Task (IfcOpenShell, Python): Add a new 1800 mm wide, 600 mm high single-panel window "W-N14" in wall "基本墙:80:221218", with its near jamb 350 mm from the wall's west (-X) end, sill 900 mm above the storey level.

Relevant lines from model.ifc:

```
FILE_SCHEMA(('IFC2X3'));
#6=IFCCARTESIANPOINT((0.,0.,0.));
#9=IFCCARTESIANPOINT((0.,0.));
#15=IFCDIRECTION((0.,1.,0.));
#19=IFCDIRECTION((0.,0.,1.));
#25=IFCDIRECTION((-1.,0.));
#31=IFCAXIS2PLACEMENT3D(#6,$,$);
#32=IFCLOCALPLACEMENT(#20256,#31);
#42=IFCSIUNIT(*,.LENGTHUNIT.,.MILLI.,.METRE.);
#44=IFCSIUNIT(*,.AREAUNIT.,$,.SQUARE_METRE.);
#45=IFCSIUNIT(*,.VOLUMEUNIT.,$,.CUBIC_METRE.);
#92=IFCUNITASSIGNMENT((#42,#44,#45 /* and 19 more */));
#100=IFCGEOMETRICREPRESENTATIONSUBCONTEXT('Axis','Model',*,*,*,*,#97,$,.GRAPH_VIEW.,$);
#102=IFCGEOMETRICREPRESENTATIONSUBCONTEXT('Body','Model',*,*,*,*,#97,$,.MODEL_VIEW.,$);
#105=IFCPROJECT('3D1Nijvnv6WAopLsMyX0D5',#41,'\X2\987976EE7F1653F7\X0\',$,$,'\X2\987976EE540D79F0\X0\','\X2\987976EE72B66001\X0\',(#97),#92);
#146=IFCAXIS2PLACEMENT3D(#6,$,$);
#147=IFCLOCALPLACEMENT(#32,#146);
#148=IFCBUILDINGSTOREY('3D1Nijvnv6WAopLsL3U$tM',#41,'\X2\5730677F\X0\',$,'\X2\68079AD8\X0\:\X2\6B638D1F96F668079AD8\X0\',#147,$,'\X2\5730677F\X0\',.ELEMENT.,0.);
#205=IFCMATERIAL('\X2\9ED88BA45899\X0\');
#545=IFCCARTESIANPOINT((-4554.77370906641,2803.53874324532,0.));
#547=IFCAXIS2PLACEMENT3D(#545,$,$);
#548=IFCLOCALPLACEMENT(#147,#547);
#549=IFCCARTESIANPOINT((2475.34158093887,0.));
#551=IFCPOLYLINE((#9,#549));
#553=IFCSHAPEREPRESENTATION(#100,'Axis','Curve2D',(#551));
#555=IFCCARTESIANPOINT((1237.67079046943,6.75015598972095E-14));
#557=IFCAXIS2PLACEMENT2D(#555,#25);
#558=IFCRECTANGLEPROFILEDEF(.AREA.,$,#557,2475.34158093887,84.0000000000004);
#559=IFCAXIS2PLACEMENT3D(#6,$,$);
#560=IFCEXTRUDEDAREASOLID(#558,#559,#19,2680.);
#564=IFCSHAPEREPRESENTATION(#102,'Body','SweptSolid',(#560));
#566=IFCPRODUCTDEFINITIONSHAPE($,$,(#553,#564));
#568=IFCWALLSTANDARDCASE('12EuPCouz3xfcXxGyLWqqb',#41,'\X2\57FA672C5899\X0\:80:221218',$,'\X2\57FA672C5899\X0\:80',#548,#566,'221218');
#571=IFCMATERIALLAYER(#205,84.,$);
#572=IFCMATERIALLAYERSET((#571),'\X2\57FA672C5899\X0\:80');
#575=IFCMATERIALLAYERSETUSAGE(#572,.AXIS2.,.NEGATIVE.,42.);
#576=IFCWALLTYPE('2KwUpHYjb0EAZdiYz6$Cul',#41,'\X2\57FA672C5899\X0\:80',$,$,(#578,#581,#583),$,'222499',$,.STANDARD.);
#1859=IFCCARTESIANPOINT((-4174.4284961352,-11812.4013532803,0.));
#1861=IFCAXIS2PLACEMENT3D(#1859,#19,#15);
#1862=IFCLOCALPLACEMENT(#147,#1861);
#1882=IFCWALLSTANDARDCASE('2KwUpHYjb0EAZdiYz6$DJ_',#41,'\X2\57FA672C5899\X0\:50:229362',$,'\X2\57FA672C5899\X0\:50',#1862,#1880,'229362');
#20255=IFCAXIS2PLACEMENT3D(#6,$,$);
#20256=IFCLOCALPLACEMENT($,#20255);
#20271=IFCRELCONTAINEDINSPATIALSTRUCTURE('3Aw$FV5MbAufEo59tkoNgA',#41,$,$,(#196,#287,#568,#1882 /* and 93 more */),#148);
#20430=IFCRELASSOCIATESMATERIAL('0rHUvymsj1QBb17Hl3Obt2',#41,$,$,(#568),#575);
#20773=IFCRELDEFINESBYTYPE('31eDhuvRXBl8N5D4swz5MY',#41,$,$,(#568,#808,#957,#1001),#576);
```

```python
import numpy as np
import ifcopenshell
import ifcopenshell.api.feature
import ifcopenshell.api.geometry
import ifcopenshell.api.root
import ifcopenshell.api.spatial
import ifcopenshell.api.type
import ifcopenshell.geom
import ifcopenshell.util.element
import ifcopenshell.util.placement
import ifcopenshell.util.representation
import ifcopenshell.util.shape
import ifcopenshell.util.unit

model = ifcopenshell.open("model.ifc")
unit_scale = ifcopenshell.util.unit.calculate_unit_scale(model)
settings = ifcopenshell.geom.settings()


def volume(element):
    """Net volume in cubic metres, openings subtracted."""
    shape = ifcopenshell.geom.create_shape(settings, element)
    return ifcopenshell.util.shape.get_volume(shape.geometry)


wall = model.by_id(568)
storey = ifcopenshell.util.element.get_container(wall, ifc_class="IfcBuildingStorey")
context = ifcopenshell.util.representation.get_context(model, "Model", "Body", "MODEL_VIEW")
before = volume(wall)

width, height, from_end, sill = 1.8, 0.6, 0.35, 0.9  # metres

# The wall runs along its own X axis, and the end named is its -X end.
wall_shape = ifcopenshell.geom.create_shape(settings, wall)
x, y, z = ifcopenshell.util.shape.get_vertices(wall_shape.geometry).T
start = x.min() + from_end
face, thickness = float(y.min()), float(y.max() - y.min())
wall_matrix = ifcopenshell.util.placement.get_local_placement(wall.ObjectPlacement)
level = ifcopenshell.util.placement.get_local_placement(storey.ObjectPlacement)[2, 3]


def in_wall(x, y):
    """Placement at x, y metres in the wall's axes, at sill height."""
    matrix = wall_matrix.copy()
    matrix[:, 3] = wall_matrix @ np.array([x / unit_scale, y / unit_scale, 0.0, 1.0])
    matrix[2, 3] = level + sill / unit_scale
    return matrix


# Opening: a box that overshoots both wall faces by 50 mm.
opening = ifcopenshell.api.root.create_entity(model, ifc_class="IfcOpeningElement")
box = ifcopenshell.api.geometry.add_wall_representation(
    model, context=context, length=width, height=height, thickness=thickness + 0.1
)
ifcopenshell.api.geometry.assign_representation(model, product=opening, representation=box)
ifcopenshell.api.geometry.edit_object_placement(model, product=opening, matrix=in_wall(start, face - 0.05), is_si=False)
ifcopenshell.api.feature.add_feature(model, feature=opening, element=wall)

window = ifcopenshell.api.root.create_entity(model, ifc_class="IfcWindow", name="W-N14")
window.OverallWidth, window.OverallHeight = width / unit_scale, height / unit_scale
body = ifcopenshell.api.geometry.add_window_representation(
    model,
    context=context,
    overall_width=window.OverallWidth,
    overall_height=window.OverallHeight,
    partition_type="SINGLE_PANEL",
)
ifcopenshell.api.geometry.assign_representation(model, product=window, representation=body)
ifcopenshell.api.spatial.assign_container(model, products=[window], relating_structure=storey)
fills = ifcopenshell.api.feature.add_filling(model, opening=opening, element=window)
fills.OwnerHistory = window.OwnerHistory  # required in IFC2X3

# IFC2X3 keeps the operation on the window style.
style = ifcopenshell.api.root.create_entity(model, ifc_class="IfcWindowStyle", name="W-N14")
style.OperationType, style.ConstructionType = "SINGLE_PANEL", "NOTDEFINED"
style.ParameterTakesPrecedence = style.Sizeable = False
ifcopenshell.api.type.assign_type(model, related_objects=[window], relating_type=style)

# Centre the window in the wall's thickness.
ifcopenshell.api.geometry.edit_object_placement(model, product=window, matrix=in_wall(start, face), is_si=False)
window_shape = ifcopenshell.geom.create_shape(settings, window)
depth = ifcopenshell.util.shape.get_vertices(window_shape.geometry)[:, 1]
offset = face + thickness / 2 - (depth.min() + depth.max()) / 2
ifcopenshell.api.geometry.edit_object_placement(model, product=window, matrix=in_wall(start, offset), is_si=False)

after = volume(wall)

print(f"wall volume {before:.3f} -> {after:.3f} m3")

model.write("model_edited.ifc")
```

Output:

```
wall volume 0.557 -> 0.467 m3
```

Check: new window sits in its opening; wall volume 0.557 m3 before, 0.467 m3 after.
